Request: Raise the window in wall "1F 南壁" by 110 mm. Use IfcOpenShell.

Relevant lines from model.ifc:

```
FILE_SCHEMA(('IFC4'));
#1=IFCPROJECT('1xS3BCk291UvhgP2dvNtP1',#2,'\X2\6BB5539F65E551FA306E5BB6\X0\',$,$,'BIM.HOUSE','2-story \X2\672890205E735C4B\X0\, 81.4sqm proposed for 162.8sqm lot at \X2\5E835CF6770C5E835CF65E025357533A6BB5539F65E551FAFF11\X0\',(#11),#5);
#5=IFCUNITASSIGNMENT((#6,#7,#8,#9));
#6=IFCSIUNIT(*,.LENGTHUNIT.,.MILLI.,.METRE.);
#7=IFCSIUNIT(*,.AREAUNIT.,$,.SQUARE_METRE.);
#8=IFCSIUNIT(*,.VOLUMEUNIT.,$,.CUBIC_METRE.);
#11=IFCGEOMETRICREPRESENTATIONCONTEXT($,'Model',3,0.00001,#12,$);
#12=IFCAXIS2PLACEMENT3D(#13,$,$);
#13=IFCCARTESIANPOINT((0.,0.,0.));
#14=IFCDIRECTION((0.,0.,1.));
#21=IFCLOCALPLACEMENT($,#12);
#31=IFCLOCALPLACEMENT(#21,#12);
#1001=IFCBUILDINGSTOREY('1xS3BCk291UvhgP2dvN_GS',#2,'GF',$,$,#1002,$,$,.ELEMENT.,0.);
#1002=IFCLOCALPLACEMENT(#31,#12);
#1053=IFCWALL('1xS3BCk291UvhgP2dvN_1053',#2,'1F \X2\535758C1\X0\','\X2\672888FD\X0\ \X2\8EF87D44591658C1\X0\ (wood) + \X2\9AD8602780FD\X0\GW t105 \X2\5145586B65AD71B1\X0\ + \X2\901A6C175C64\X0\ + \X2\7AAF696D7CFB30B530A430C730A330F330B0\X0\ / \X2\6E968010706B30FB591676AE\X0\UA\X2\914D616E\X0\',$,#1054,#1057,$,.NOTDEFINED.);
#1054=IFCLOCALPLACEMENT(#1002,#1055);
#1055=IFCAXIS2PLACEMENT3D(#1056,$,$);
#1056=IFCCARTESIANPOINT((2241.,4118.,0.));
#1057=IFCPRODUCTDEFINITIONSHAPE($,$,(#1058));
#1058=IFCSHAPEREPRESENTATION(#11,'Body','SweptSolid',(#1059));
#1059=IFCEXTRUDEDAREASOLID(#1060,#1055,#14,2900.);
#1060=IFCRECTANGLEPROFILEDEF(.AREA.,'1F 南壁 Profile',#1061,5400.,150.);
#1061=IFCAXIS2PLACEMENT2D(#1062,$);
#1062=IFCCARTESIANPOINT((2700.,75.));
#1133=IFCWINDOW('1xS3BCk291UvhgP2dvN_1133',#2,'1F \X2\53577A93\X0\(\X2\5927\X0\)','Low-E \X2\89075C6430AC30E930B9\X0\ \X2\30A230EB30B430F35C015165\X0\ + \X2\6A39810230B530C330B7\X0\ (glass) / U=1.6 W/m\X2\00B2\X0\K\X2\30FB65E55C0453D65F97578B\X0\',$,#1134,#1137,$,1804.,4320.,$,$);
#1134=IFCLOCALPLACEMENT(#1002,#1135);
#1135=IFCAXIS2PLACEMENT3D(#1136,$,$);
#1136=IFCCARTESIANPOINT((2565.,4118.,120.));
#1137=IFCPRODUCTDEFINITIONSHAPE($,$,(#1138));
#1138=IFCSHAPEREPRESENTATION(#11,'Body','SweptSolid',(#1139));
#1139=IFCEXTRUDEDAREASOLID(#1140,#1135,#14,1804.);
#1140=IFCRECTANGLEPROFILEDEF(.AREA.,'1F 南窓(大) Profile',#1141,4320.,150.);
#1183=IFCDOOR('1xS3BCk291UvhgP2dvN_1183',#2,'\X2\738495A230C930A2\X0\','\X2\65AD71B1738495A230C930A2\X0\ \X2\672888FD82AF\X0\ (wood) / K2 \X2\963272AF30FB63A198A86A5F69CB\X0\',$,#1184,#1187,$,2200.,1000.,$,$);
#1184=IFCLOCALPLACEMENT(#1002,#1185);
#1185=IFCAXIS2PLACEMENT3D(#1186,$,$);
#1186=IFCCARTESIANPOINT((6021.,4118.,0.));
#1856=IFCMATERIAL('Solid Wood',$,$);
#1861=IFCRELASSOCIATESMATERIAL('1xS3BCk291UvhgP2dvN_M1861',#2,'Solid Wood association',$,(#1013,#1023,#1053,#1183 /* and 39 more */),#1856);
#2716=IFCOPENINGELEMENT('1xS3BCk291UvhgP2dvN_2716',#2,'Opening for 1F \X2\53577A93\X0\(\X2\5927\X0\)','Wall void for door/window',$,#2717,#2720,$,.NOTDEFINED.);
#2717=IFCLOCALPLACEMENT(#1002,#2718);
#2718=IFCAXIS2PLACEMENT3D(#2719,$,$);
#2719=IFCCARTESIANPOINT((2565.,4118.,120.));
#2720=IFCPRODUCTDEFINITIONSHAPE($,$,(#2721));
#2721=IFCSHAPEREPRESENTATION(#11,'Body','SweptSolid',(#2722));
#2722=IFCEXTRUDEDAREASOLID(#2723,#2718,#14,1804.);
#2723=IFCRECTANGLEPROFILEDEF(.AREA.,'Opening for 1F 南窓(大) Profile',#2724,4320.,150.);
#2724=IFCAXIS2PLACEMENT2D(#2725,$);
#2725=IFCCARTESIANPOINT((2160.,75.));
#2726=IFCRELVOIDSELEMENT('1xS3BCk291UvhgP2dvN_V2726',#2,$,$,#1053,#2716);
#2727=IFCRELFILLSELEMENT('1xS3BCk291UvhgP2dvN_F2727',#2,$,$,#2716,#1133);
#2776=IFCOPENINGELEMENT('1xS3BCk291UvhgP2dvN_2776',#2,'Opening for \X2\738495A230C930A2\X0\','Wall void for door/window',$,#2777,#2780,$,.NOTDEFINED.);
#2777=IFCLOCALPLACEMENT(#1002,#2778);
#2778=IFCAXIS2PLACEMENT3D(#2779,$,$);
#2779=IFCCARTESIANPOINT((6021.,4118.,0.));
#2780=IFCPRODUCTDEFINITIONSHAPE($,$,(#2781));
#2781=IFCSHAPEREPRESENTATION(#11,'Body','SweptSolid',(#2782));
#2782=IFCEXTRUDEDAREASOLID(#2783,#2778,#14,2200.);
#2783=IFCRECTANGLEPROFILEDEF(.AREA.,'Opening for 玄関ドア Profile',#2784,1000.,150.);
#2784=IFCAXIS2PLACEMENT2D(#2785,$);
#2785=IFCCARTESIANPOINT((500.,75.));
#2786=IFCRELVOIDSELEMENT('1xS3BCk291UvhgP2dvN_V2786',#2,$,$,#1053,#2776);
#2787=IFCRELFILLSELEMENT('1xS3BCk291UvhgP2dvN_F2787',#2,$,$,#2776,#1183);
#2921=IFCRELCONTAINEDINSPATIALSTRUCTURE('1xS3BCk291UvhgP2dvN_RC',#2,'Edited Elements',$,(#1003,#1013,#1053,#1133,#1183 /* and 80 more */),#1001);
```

```python
import numpy as np
import ifcopenshell
import ifcopenshell.api.geometry
import ifcopenshell.util.placement
import ifcopenshell.util.unit

model = ifcopenshell.open("model.ifc")
unit_scale = ifcopenshell.util.unit.calculate_unit_scale(model)

window = model.by_guid("1xS3BCk291UvhgP2dvN_1133")
opening = window.FillsVoids[0].RelatingOpeningElement
dz = 0.11 / unit_scale

shift = np.array([0.0, 0.0, dz])
# The window is not placed relative to its opening, so move both.
for product in (opening, window):
    matrix = ifcopenshell.util.placement.get_local_placement(product.ObjectPlacement)
    matrix[:3, 3] += shift
    ifcopenshell.api.geometry.edit_object_placement(model, product=product, matrix=matrix, is_si=False)

print(f"moved by {dz * unit_scale:+.3f} m")

model.write("model_updated.ifc")
```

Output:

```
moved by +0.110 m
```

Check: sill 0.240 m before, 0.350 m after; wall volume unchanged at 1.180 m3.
